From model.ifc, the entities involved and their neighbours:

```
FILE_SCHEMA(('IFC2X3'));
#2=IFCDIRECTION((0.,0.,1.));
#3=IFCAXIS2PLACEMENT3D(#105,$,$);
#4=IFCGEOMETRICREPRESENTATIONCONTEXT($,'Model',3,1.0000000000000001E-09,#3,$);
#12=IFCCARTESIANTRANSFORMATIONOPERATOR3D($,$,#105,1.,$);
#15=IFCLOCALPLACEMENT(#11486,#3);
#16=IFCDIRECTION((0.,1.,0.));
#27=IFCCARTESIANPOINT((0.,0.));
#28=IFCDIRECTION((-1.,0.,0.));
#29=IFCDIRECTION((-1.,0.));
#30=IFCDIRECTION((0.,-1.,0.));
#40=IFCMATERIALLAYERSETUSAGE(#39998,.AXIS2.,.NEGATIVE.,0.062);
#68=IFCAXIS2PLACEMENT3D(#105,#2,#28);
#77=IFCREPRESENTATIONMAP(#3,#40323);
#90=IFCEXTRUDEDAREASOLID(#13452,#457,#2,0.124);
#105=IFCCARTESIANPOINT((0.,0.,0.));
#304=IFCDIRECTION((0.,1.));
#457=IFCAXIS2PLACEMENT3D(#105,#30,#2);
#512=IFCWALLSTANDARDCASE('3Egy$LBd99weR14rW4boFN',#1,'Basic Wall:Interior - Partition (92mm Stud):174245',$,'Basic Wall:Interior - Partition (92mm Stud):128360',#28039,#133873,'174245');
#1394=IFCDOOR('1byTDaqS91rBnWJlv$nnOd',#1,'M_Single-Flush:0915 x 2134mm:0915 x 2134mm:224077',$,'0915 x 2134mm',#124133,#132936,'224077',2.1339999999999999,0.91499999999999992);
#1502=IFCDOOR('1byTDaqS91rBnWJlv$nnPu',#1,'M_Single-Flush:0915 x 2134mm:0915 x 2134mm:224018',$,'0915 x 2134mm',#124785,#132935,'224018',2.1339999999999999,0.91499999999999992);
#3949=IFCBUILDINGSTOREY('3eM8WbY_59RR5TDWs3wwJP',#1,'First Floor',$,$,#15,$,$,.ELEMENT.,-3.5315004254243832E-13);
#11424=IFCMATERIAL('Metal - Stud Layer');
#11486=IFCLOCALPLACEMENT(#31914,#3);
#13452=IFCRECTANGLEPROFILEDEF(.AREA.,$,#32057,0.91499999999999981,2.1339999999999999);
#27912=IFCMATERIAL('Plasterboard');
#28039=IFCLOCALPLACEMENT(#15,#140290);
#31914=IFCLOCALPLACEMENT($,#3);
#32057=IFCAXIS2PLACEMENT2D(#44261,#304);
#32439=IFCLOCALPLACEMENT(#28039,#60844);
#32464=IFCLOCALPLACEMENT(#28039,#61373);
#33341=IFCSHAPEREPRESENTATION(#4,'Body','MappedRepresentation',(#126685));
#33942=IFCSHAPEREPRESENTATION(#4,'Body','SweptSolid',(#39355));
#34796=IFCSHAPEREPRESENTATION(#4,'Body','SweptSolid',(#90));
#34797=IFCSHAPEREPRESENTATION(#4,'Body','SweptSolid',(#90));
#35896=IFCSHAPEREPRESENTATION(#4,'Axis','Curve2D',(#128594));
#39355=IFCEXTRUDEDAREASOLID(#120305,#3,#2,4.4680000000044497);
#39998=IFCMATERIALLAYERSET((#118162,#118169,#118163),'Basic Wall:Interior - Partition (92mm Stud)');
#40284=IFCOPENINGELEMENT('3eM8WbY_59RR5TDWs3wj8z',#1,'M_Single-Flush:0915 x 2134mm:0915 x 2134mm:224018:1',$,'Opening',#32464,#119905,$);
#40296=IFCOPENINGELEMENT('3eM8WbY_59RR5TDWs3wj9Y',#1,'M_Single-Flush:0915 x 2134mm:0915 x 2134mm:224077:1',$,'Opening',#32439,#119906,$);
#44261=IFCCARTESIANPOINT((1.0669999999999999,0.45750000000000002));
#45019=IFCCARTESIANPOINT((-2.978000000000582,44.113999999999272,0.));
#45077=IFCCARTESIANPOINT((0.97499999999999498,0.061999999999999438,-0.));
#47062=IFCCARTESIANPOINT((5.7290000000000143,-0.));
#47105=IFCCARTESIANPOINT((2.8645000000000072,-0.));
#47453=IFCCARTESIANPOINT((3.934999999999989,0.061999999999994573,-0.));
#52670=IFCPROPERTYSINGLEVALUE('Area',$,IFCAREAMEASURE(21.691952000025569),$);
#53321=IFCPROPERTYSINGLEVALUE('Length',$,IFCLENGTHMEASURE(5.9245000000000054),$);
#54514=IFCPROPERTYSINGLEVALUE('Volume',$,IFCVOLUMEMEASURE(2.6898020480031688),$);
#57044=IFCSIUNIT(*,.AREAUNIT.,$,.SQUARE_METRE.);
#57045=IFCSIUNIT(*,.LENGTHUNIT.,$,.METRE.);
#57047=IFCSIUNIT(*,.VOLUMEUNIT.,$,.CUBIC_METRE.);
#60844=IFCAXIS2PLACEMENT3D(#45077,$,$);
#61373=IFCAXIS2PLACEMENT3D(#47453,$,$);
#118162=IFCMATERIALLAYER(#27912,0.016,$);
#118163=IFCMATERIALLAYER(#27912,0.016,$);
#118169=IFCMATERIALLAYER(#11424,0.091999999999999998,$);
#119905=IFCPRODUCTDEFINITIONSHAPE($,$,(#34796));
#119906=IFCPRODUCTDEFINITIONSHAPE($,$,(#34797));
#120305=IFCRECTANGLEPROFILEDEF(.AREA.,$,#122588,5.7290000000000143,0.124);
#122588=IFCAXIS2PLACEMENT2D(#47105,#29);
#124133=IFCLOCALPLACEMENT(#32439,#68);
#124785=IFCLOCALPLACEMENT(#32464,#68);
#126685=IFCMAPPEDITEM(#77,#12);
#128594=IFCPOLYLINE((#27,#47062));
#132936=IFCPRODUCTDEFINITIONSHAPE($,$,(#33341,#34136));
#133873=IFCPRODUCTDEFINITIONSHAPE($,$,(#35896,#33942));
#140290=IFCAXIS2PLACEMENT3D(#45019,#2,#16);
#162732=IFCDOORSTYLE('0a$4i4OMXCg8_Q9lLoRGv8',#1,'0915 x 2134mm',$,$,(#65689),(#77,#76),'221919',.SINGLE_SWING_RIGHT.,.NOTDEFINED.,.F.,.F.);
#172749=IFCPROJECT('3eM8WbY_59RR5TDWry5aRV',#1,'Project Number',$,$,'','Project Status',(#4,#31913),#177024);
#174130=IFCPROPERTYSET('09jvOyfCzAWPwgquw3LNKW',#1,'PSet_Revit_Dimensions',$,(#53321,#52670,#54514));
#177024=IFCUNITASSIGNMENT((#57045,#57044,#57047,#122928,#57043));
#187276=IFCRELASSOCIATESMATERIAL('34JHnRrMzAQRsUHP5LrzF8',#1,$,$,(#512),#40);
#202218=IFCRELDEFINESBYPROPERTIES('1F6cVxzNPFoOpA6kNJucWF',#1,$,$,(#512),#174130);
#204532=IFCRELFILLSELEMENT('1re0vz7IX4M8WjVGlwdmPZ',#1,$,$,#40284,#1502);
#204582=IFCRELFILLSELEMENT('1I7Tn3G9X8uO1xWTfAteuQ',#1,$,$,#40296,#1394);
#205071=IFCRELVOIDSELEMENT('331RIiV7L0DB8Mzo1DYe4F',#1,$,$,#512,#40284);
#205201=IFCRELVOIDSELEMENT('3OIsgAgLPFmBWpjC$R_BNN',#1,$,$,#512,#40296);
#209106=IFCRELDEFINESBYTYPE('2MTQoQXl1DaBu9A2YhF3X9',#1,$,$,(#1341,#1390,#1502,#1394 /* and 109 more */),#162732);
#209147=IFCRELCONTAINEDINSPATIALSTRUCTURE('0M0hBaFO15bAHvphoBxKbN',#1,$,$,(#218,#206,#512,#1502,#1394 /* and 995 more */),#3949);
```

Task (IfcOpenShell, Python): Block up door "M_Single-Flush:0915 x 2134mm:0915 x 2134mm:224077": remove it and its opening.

```python
import ifcopenshell
import ifcopenshell.api.feature
import ifcopenshell.api.pset
import ifcopenshell.api.root
import ifcopenshell.geom
import ifcopenshell.util.element
import ifcopenshell.util.shape
import ifcopenshell.util.unit

model = ifcopenshell.open("model.ifc")
area_scale = ifcopenshell.util.unit.calculate_unit_scale(model, "AREAUNIT")
volume_scale = ifcopenshell.util.unit.calculate_unit_scale(model, "VOLUMEUNIT")
settings = ifcopenshell.geom.settings()


def volume(element):
    """Net volume in cubic metres, openings subtracted."""
    shape = ifcopenshell.geom.create_shape(settings, element)
    return ifcopenshell.util.shape.get_volume(shape.geometry)


door = model.by_guid("1byTDaqS91rBnWJlv$nnOd")
opening = door.FillsVoids[0].RelatingOpeningElement
wall = opening.VoidsElements[0].RelatingBuildingElement
before = volume(wall)

ifcopenshell.api.root.remove_product(model, product=door)
ifcopenshell.api.feature.remove_feature(model, feature=opening)

after = volume(wall)
thickness = 0.124  # wall thickness in metres

# Update the wall's stored quantities.
pset = model.by_id(ifcopenshell.util.element.get_pset(wall, "PSet_Revit_Dimensions", should_inherit=False)["id"])
ifcopenshell.api.pset.edit_pset(model, pset=pset, properties={
    "Area": model.create_entity("IfcAreaMeasure", after / thickness / area_scale),
    "Volume": model.create_entity("IfcVolumeMeasure", after / volume_scale),
})

print(f"wall volume {before:.3f} -> {after:.3f} m3")

model.write("model_rev.ifc")
```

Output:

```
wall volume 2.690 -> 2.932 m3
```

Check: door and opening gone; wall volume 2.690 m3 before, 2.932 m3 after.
